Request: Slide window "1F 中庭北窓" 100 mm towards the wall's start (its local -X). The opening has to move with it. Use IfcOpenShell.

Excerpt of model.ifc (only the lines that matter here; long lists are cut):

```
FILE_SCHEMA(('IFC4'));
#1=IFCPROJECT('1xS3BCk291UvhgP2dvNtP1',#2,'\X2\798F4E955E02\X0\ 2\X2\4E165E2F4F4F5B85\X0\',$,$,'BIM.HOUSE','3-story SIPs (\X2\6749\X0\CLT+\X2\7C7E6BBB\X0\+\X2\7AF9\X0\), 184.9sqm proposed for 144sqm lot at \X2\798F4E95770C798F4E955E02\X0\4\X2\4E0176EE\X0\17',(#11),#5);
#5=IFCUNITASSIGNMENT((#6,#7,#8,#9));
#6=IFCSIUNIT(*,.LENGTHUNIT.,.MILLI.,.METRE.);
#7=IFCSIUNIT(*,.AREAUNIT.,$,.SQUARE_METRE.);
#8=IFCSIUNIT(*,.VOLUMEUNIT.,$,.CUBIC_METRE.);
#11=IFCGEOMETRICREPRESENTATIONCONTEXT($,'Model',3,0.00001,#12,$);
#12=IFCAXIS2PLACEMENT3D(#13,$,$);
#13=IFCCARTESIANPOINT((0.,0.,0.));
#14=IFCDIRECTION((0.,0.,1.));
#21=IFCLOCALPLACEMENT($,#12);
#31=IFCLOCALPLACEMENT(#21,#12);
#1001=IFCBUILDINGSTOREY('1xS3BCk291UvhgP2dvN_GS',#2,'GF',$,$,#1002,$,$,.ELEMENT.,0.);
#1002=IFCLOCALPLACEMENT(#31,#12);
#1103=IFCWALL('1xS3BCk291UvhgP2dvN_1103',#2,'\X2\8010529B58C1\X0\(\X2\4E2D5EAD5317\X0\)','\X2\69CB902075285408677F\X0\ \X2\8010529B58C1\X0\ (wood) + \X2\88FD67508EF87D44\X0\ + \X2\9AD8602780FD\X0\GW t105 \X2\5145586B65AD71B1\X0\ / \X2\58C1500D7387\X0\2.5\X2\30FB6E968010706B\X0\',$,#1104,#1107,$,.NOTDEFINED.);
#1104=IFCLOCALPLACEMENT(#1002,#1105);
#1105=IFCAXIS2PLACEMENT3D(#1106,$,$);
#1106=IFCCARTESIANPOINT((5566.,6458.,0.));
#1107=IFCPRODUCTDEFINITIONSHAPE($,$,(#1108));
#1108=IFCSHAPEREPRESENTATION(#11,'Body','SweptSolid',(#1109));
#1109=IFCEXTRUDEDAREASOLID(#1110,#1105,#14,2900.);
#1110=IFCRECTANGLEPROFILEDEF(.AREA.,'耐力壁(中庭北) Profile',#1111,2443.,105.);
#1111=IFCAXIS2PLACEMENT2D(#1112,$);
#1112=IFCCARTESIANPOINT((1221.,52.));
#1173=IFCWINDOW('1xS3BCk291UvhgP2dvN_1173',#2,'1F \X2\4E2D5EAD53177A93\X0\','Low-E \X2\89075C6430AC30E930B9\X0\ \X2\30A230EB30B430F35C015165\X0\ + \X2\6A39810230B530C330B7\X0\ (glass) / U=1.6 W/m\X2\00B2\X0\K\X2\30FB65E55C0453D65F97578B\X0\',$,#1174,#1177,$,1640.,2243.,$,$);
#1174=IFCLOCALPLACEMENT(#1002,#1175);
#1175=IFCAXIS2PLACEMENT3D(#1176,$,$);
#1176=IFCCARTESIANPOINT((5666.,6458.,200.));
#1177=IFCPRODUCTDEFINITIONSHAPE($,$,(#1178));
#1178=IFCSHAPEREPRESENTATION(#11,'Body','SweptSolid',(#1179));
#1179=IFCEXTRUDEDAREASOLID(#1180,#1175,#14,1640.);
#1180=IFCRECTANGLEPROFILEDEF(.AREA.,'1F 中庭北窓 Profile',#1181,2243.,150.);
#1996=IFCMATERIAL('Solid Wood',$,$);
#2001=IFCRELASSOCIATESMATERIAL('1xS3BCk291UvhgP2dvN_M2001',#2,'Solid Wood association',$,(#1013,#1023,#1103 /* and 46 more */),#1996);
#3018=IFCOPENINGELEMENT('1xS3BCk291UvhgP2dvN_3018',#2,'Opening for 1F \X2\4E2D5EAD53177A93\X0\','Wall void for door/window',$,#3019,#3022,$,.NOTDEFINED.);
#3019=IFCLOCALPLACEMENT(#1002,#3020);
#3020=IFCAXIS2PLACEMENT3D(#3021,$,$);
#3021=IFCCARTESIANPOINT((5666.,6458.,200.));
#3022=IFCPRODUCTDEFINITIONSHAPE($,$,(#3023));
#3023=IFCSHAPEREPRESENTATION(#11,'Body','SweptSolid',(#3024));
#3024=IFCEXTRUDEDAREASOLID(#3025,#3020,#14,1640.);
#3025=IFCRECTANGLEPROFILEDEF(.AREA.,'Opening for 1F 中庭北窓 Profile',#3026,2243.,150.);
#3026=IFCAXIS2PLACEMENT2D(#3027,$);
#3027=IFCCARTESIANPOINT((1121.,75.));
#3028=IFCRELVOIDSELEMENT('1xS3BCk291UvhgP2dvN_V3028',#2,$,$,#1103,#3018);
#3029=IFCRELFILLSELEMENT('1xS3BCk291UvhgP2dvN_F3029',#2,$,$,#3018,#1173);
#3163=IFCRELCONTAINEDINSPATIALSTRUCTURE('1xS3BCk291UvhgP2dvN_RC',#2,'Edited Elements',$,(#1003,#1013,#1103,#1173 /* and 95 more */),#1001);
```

```python
import ifcopenshell
import ifcopenshell.api.geometry
import ifcopenshell.util.placement

model = ifcopenshell.open("model.ifc")

window = model.by_guid("1xS3BCk291UvhgP2dvN_1173")
opening = window.FillsVoids[0].RelatingOpeningElement
wall = opening.VoidsElements[0].RelatingBuildingElement

wall_matrix = ifcopenshell.util.placement.get_local_placement(wall.ObjectPlacement)
shift = wall_matrix[:3, 0] * -100.0
before = ifcopenshell.util.placement.get_local_placement(window.ObjectPlacement)[:3, 3].copy()

# The window is not placed relative to its opening, so move both.
for product in (opening, window):
    matrix = ifcopenshell.util.placement.get_local_placement(product.ObjectPlacement)
    matrix[:3, 3] += shift
    ifcopenshell.api.geometry.edit_object_placement(model, product=product, matrix=matrix, is_si=False)

after = ifcopenshell.util.placement.get_local_placement(window.ObjectPlacement)[:3, 3]
print("window moved by", (after - before).round(3) + 0.0)

model.write("model_updated.ifc")
```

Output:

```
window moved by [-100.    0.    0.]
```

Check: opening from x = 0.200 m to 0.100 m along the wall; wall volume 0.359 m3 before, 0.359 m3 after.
